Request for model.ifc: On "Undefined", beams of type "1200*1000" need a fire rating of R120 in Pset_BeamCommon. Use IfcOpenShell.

First a look at what the model holds.

```python
import ifcopenshell
import ifcopenshell.util.element

model = ifcopenshell.open("model.ifc")
print(model.schema)
storey = next(s for s in model.by_type("IfcBuildingStorey") if s.Name == "Undefined")
beams = [e for e in ifcopenshell.util.element.get_decomposition(storey) if e.is_a("IfcBeam")]
seen = {}
for e in beams:
    element_type = ifcopenshell.util.element.get_type(e)
    key = (element_type.Name if element_type != e and element_type else None, ifcopenshell.util.element.get_pset(e, "Pset_BeamCommon", "FireRating"))
    seen[key] = seen.get(key, 0) + 1
for (name, value), count in sorted(seen.items(), key=str):
    print(count, "x", name, "|", value)
```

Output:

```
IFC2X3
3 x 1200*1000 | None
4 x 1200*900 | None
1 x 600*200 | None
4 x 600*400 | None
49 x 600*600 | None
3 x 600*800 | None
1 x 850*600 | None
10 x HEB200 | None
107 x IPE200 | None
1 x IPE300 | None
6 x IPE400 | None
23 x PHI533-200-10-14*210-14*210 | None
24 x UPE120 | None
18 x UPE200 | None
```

```python
import ifcopenshell
import ifcopenshell.api.pset
import ifcopenshell.util.element

model = ifcopenshell.open("model.ifc")

storey = next(s for s in model.by_type("IfcBuildingStorey") if s.Name == "Undefined")
beams = [e for e in ifcopenshell.util.element.get_decomposition(storey) if e.is_a("IfcBeam")]

count = 0
for e in beams:
    element_type = ifcopenshell.util.element.get_type(e)
    if element_type in (None, e) or element_type.Name != "1200*1000":
        continue
    found = ifcopenshell.util.element.get_pset(e, "Pset_BeamCommon", should_inherit=False)
    if found:
        pset = model.by_id(found["id"])
        if len(ifcopenshell.util.element.get_elements_by_pset(pset)) > 1:
            pset = ifcopenshell.api.pset.unshare_pset(model, products=[e], pset=pset)[0]
    else:
        pset = ifcopenshell.api.pset.add_pset(model, product=e, name="Pset_BeamCommon")
    ifcopenshell.api.pset.edit_pset(model, pset=pset, properties={"FireRating": "R120"})
    count += 1

print(count, "beams updated")

model.write("model_updated.ifc")
```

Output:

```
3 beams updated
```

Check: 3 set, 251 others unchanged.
